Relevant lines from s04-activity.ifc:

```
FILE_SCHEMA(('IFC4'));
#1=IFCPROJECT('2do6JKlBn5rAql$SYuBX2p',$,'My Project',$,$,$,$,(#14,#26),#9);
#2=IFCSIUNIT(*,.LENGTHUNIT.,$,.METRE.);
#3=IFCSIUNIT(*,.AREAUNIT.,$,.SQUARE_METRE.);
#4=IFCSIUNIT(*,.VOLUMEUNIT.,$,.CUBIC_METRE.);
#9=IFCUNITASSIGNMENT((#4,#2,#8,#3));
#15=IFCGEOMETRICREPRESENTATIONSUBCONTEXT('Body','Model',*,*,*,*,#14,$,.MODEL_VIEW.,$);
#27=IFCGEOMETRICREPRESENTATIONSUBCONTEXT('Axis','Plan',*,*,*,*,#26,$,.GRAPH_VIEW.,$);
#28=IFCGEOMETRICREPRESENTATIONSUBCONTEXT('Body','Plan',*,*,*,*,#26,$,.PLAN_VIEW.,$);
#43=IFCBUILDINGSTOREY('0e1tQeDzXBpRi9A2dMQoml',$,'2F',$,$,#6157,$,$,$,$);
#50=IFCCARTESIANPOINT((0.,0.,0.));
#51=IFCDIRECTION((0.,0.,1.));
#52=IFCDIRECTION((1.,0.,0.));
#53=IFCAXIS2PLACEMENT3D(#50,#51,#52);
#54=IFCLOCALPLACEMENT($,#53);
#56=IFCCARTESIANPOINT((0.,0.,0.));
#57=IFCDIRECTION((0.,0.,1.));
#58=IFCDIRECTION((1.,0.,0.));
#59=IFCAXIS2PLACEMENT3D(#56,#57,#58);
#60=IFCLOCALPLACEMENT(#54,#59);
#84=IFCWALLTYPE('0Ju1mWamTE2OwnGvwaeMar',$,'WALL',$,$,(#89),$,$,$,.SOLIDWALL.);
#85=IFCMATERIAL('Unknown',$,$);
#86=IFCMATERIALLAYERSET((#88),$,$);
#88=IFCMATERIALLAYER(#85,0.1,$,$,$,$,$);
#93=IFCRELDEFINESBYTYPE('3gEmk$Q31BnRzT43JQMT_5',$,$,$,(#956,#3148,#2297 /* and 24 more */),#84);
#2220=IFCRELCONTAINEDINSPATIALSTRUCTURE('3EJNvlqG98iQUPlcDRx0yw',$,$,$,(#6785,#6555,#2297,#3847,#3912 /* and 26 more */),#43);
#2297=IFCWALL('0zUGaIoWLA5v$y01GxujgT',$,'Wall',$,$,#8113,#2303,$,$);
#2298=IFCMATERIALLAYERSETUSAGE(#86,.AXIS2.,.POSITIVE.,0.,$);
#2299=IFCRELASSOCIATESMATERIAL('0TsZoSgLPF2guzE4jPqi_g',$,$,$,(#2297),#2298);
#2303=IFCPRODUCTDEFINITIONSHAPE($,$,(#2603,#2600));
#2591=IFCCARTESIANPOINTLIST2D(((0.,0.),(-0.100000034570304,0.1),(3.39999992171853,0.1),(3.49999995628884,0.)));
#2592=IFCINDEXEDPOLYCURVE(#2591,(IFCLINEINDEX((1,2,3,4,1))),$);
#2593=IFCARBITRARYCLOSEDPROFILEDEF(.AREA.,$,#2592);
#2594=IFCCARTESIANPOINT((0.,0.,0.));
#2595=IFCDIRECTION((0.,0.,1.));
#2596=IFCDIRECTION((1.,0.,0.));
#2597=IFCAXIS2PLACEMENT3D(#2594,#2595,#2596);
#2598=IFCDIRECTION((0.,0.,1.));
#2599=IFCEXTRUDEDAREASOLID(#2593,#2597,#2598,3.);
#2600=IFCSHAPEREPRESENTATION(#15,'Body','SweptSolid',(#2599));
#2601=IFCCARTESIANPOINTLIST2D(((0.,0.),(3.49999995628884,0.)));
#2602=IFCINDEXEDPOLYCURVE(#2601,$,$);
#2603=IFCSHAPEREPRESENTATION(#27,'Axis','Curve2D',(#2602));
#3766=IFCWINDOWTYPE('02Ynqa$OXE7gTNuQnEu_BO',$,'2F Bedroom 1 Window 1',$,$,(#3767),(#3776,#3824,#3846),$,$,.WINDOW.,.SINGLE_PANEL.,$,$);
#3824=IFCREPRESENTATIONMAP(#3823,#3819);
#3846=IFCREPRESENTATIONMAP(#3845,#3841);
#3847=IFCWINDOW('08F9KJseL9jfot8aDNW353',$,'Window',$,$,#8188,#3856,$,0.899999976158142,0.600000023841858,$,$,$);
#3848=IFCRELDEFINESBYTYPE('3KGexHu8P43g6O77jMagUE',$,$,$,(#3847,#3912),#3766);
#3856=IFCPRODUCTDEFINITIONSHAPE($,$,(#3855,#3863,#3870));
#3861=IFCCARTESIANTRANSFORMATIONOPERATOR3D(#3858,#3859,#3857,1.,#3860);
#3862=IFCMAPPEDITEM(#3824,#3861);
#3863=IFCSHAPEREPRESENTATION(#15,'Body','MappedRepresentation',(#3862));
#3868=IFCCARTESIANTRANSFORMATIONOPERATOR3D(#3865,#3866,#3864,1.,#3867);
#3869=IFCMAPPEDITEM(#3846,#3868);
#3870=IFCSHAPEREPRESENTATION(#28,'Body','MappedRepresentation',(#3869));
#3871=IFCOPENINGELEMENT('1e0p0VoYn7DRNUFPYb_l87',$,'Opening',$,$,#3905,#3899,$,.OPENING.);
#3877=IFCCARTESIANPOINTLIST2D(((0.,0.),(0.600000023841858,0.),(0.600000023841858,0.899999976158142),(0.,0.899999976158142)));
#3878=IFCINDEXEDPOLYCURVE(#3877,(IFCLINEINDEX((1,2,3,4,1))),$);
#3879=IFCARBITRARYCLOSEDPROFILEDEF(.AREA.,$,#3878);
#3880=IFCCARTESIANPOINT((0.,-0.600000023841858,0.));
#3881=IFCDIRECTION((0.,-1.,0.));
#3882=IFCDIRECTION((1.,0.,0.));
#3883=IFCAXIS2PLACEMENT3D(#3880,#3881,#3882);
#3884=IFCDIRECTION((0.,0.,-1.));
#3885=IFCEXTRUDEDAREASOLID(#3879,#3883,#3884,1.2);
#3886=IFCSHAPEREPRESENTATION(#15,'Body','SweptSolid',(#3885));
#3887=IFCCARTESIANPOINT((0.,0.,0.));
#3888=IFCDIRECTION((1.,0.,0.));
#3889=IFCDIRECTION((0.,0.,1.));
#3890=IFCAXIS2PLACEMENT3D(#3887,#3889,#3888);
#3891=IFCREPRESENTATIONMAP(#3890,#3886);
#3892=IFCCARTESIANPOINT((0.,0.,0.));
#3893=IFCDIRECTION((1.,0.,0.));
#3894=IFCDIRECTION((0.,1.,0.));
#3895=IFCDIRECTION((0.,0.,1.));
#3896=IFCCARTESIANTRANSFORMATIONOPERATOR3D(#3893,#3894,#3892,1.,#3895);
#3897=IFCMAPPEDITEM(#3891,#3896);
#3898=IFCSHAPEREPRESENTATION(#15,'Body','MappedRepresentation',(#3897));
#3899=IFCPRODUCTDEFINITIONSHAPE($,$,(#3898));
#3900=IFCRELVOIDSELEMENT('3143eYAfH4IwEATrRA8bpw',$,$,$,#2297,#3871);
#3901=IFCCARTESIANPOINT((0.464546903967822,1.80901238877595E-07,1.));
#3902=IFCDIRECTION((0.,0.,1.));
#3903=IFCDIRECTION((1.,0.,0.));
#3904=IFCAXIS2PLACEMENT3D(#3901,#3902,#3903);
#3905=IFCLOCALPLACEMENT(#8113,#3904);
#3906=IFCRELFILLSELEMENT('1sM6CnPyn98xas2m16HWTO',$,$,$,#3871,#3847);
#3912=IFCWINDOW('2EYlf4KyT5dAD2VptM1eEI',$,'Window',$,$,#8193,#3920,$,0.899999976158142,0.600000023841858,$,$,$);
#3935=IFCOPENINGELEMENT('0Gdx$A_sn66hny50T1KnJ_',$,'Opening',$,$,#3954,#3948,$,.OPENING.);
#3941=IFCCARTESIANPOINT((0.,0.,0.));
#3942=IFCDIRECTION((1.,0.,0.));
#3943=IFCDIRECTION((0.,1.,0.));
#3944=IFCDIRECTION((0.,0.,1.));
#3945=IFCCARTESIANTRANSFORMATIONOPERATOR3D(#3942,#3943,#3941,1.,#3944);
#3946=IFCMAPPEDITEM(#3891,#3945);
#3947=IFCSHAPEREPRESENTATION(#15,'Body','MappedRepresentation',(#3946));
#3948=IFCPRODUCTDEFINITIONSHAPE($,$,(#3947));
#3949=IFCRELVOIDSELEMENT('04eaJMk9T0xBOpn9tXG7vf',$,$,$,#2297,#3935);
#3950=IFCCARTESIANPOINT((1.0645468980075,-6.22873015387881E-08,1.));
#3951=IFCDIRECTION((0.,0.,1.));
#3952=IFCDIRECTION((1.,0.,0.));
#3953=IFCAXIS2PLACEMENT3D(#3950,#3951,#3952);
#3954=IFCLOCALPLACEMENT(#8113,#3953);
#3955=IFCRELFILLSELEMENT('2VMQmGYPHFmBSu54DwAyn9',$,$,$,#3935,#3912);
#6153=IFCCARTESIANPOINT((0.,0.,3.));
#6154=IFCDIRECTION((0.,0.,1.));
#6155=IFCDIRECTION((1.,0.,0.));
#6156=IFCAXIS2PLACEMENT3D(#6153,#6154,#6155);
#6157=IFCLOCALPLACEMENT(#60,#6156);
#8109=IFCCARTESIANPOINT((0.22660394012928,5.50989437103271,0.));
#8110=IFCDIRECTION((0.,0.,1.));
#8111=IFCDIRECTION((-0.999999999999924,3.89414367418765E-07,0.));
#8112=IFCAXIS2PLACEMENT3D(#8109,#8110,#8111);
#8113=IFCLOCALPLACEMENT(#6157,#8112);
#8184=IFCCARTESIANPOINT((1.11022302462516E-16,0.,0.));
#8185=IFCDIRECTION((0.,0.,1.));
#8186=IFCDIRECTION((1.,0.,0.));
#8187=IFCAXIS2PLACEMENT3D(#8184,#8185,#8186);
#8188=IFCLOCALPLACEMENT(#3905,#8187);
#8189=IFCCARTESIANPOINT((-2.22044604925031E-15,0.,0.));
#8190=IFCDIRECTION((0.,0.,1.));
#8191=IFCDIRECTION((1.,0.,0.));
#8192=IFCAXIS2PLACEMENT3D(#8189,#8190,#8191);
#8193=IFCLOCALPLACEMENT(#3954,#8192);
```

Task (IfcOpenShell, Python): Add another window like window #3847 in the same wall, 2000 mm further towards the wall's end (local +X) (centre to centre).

```python
import ifcopenshell
import ifcopenshell.api.feature
import ifcopenshell.api.geometry
import ifcopenshell.api.root
import ifcopenshell.geom
import ifcopenshell.util.element
import ifcopenshell.util.placement
import ifcopenshell.util.shape
import ifcopenshell.util.unit

model = ifcopenshell.open("s04-activity.ifc")
unit_scale = ifcopenshell.util.unit.calculate_unit_scale(model)
settings = ifcopenshell.geom.settings()


def volume(element):
    """Net volume in cubic metres, openings subtracted."""
    shape = ifcopenshell.geom.create_shape(settings, element)
    return ifcopenshell.util.shape.get_volume(shape.geometry)


window = model.by_guid("08F9KJseL9jfot8aDNW353")
opening = window.FillsVoids[0].RelatingOpeningElement
wall = opening.VoidsElements[0].RelatingBuildingElement
before = volume(wall)
shift = ifcopenshell.util.placement.get_local_placement(wall.ObjectPlacement)[:3, 0] * 2 / unit_scale

# copy_class copies the void relationship, type, container and properties, but no geometry.
new_opening = ifcopenshell.api.root.copy_class(model, product=opening)
new_opening.Representation = ifcopenshell.util.element.copy_deep(
    model, opening.Representation, exclude=["IfcGeometricRepresentationContext", "IfcRepresentationMap"]
)
new_window = ifcopenshell.api.root.copy_class(model, product=window)
new_window.Representation = ifcopenshell.util.element.copy_deep(
    model, window.Representation, exclude=["IfcGeometricRepresentationContext", "IfcRepresentationMap"]
)
ifcopenshell.api.feature.add_filling(model, opening=new_opening, element=new_window)

for old, new in ((opening, new_opening), (window, new_window)):
    matrix = ifcopenshell.util.placement.get_local_placement(old.ObjectPlacement)
    matrix[:3, 3] += shift
    ifcopenshell.api.geometry.edit_object_placement(model, product=new, matrix=matrix, is_si=False)

after = volume(wall)

print(f"wall volume {before:.3f} -> {after:.3f} m3")

model.write("s04-activity_edited.ifc")
```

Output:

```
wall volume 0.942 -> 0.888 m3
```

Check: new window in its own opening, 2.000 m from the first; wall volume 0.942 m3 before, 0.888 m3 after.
